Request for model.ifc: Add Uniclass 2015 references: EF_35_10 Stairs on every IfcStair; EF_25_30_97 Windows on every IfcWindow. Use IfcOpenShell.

First a look at what the model holds.

```python
import ifcopenshell

model = ifcopenshell.open("model.ifc")
print(model.schema)
print("classifications:", [c.Name for c in model.by_type("IfcClassification")])
for ifc_class in ("IfcDoor", "IfcRoof", "IfcStair", "IfcWall", "IfcWindow"):
    print(ifc_class, len(model.by_type(ifc_class)))
```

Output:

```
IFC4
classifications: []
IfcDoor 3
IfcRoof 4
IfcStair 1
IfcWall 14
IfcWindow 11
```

```python
import ifcopenshell
import ifcopenshell.api.classification

model = ifcopenshell.open("model.ifc")

system = ifcopenshell.api.classification.add_classification(model, classification="Uniclass 2015")

codes = {
    "IfcStair": ("EF_35_10", "Stairs"),
    "IfcWindow": ("EF_25_30_97", "Windows"),
}
for ifc_class, (code, name) in codes.items():
    products = model.by_type(ifc_class)
    ifcopenshell.api.classification.add_reference(
        model, products=products, classification=system, identification=code, name=name
    )
    print(code, len(products))

model.write("model_edited.ifc")
```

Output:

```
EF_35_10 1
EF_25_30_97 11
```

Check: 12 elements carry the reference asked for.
